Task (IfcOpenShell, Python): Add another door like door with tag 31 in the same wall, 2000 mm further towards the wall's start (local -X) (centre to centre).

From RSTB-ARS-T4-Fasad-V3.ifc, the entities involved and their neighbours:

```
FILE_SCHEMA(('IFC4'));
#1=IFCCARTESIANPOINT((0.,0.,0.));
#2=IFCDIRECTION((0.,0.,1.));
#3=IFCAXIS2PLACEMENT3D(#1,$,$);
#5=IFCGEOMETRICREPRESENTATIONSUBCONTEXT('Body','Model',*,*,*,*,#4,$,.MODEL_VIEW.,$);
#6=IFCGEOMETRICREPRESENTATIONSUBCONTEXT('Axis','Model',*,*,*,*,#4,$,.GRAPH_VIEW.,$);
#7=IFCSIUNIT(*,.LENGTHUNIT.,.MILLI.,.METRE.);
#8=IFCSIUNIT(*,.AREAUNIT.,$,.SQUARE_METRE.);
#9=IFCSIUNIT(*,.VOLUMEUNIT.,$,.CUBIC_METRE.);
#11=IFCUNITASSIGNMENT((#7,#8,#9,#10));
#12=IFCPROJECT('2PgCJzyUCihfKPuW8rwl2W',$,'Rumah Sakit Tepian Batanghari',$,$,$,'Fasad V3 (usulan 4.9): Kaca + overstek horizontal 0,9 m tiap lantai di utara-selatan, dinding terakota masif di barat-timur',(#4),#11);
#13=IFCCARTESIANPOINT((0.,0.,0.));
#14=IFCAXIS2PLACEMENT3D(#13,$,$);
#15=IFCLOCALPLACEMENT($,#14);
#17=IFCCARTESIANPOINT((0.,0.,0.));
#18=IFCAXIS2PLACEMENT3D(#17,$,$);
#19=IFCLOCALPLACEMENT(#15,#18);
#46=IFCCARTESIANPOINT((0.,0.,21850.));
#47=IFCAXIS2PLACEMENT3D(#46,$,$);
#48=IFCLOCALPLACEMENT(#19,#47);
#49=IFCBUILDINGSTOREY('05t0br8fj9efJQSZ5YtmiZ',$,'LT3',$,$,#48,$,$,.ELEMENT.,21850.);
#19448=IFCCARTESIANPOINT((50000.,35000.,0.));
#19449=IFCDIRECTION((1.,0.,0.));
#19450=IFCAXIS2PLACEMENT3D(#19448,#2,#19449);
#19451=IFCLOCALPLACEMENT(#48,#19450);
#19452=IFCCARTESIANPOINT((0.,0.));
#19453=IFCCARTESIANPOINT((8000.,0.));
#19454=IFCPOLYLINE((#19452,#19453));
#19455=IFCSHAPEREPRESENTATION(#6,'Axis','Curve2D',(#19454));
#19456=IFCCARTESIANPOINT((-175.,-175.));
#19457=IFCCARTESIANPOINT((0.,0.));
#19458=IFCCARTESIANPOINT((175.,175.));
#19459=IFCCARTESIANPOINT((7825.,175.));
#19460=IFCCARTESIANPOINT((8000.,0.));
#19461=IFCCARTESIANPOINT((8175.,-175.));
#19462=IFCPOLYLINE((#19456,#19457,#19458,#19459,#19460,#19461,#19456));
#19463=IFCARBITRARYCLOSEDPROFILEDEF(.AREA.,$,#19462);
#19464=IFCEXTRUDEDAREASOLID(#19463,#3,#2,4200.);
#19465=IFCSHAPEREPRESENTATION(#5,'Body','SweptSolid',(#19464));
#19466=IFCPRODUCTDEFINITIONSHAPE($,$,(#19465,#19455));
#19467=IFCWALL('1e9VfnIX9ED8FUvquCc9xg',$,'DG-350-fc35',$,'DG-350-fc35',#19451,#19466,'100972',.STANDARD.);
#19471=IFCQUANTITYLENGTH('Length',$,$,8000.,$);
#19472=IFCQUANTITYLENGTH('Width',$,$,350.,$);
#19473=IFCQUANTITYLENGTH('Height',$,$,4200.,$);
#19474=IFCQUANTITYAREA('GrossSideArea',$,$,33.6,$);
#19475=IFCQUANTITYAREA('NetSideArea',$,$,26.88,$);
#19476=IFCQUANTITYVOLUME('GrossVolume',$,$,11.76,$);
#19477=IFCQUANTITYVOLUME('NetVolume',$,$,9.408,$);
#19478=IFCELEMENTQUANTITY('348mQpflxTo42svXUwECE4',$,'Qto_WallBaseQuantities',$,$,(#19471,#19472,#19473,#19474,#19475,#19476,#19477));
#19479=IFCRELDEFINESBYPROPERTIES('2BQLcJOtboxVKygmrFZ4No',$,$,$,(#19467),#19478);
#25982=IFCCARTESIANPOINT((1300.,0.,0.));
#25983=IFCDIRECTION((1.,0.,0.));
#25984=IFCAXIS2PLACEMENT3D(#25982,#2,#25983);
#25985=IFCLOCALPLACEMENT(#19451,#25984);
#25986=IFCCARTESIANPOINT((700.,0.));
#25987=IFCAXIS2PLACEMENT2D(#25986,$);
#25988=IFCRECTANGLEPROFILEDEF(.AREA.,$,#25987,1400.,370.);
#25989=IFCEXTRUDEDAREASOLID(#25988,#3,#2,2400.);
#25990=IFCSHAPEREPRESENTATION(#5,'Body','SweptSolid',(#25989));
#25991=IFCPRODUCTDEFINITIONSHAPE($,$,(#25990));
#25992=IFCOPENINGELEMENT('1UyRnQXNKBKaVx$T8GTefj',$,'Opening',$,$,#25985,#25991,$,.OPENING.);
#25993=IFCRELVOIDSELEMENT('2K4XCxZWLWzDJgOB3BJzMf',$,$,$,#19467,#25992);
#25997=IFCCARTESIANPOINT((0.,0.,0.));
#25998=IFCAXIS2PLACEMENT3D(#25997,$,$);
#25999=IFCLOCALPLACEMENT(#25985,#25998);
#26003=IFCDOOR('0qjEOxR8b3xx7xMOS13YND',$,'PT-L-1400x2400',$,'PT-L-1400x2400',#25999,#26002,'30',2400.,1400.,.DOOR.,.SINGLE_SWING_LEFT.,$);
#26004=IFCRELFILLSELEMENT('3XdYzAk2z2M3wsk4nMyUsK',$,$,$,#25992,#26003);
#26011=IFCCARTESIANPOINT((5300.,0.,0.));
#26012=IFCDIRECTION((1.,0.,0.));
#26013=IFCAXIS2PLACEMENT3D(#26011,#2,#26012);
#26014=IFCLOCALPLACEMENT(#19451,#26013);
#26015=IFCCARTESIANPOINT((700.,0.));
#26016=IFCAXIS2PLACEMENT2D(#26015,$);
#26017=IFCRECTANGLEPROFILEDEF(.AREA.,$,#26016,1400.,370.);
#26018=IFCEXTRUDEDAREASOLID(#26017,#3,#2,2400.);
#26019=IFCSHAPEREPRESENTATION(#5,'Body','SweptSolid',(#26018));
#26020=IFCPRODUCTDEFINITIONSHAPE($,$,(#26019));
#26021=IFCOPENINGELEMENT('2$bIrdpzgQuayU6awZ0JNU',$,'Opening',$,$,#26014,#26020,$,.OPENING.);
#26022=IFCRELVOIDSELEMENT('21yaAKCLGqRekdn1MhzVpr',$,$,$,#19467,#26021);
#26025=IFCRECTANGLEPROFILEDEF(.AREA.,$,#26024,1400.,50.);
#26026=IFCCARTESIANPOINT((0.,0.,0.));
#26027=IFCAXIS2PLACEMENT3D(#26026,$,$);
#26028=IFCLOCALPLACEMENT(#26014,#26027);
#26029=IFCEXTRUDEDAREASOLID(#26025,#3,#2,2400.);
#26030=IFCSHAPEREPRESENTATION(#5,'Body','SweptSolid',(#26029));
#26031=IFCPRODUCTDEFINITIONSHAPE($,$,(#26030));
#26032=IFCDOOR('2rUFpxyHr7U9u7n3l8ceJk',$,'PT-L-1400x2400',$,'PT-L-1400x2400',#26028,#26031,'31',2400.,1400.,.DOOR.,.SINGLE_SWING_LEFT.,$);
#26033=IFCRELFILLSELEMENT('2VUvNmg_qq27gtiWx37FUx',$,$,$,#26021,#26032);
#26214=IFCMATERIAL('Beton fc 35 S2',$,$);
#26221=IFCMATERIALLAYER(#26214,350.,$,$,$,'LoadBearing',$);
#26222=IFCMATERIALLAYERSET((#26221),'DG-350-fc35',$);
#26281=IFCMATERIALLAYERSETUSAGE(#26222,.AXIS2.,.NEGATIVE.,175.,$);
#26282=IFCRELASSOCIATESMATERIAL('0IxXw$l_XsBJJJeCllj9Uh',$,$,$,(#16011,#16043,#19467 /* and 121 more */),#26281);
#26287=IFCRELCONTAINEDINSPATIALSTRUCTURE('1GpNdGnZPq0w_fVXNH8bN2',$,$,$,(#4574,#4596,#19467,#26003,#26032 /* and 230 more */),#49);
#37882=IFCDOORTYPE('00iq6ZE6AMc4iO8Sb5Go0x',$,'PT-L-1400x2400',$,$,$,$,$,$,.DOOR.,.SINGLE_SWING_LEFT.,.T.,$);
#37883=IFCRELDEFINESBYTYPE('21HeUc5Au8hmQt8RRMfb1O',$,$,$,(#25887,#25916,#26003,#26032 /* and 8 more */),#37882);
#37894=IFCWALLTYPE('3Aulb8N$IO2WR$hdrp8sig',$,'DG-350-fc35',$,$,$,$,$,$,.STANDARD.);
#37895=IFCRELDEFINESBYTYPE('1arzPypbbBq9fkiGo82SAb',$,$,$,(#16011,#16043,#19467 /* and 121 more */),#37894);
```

```python
import ifcopenshell
import ifcopenshell.api.feature
import ifcopenshell.api.geometry
import ifcopenshell.api.pset
import ifcopenshell.api.root
import ifcopenshell.geom
import ifcopenshell.util.element
import ifcopenshell.util.placement
import ifcopenshell.util.shape
import ifcopenshell.util.unit

model = ifcopenshell.open("RSTB-ARS-T4-Fasad-V3.ifc")
area_scale = ifcopenshell.util.unit.calculate_unit_scale(model, "AREAUNIT")
volume_scale = ifcopenshell.util.unit.calculate_unit_scale(model, "VOLUMEUNIT")
settings = ifcopenshell.geom.settings()


def volume(element):
    """Net volume in cubic metres, openings subtracted."""
    shape = ifcopenshell.geom.create_shape(settings, element)
    return ifcopenshell.util.shape.get_volume(shape.geometry)


door = model.by_guid("2rUFpxyHr7U9u7n3l8ceJk")
opening = door.FillsVoids[0].RelatingOpeningElement
wall = opening.VoidsElements[0].RelatingBuildingElement
before = volume(wall)
shift = ifcopenshell.util.placement.get_local_placement(wall.ObjectPlacement)[:3, 0] * -2000.0

# copy_class copies the void relationship, type, container and properties, but no geometry.
new_opening = ifcopenshell.api.root.copy_class(model, product=opening)
new_opening.Representation = ifcopenshell.util.element.copy_deep(
    model, opening.Representation, exclude=["IfcGeometricRepresentationContext", "IfcRepresentationMap"]
)
new_door = ifcopenshell.api.root.copy_class(model, product=door)
new_door.Representation = ifcopenshell.util.element.copy_deep(
    model, door.Representation, exclude=["IfcGeometricRepresentationContext", "IfcRepresentationMap"]
)
new_door.Tag = None
ifcopenshell.api.feature.add_filling(model, opening=new_opening, element=new_door)

for old, new in ((opening, new_opening), (door, new_door)):
    matrix = ifcopenshell.util.placement.get_local_placement(old.ObjectPlacement)
    matrix[:3, 3] += shift
    ifcopenshell.api.geometry.edit_object_placement(model, product=new, matrix=matrix, is_si=False)

after = volume(wall)
thickness = 0.35  # wall thickness in metres

# Update the wall's stored quantities.
qto = model.by_id(ifcopenshell.util.element.get_pset(wall, "Qto_WallBaseQuantities", should_inherit=False)["id"])
ifcopenshell.api.pset.edit_qto(model, qto=qto, properties={
    "NetSideArea": after / thickness / area_scale,
    "NetVolume": after / volume_scale,
})

print(f"wall volume {before:.3f} -> {after:.3f} m3")

model.write("RSTB-ARS-T4-Fasad-V3_edited.ifc")
```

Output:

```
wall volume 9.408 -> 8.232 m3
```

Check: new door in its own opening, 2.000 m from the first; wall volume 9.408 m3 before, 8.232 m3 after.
